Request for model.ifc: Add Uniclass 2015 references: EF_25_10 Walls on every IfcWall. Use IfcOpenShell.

First a look at what the model holds.

```python
import ifcopenshell

model = ifcopenshell.open("model.ifc")
print(model.schema)
print("classifications:", [c.Name for c in model.by_type("IfcClassification")])
for ifc_class in ("IfcDoor", "IfcRoof", "IfcStair", "IfcWall", "IfcWindow"):
    print(ifc_class, len(model.by_type(ifc_class)))
```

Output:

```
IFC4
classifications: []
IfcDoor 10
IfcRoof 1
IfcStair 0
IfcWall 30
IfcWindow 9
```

```python
import ifcopenshell
import ifcopenshell.api.classification

model = ifcopenshell.open("model.ifc")

system = ifcopenshell.api.classification.add_classification(model, classification="Uniclass 2015")

codes = {
    "IfcWall": ("EF_25_10", "Walls"),
}
for ifc_class, (code, name) in codes.items():
    products = model.by_type(ifc_class)
    ifcopenshell.api.classification.add_reference(
        model, products=products, classification=system, identification=code, name=name
    )
    print(code, len(products))

model.write("model_updated.ifc")
```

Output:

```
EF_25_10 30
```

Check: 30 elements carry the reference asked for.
